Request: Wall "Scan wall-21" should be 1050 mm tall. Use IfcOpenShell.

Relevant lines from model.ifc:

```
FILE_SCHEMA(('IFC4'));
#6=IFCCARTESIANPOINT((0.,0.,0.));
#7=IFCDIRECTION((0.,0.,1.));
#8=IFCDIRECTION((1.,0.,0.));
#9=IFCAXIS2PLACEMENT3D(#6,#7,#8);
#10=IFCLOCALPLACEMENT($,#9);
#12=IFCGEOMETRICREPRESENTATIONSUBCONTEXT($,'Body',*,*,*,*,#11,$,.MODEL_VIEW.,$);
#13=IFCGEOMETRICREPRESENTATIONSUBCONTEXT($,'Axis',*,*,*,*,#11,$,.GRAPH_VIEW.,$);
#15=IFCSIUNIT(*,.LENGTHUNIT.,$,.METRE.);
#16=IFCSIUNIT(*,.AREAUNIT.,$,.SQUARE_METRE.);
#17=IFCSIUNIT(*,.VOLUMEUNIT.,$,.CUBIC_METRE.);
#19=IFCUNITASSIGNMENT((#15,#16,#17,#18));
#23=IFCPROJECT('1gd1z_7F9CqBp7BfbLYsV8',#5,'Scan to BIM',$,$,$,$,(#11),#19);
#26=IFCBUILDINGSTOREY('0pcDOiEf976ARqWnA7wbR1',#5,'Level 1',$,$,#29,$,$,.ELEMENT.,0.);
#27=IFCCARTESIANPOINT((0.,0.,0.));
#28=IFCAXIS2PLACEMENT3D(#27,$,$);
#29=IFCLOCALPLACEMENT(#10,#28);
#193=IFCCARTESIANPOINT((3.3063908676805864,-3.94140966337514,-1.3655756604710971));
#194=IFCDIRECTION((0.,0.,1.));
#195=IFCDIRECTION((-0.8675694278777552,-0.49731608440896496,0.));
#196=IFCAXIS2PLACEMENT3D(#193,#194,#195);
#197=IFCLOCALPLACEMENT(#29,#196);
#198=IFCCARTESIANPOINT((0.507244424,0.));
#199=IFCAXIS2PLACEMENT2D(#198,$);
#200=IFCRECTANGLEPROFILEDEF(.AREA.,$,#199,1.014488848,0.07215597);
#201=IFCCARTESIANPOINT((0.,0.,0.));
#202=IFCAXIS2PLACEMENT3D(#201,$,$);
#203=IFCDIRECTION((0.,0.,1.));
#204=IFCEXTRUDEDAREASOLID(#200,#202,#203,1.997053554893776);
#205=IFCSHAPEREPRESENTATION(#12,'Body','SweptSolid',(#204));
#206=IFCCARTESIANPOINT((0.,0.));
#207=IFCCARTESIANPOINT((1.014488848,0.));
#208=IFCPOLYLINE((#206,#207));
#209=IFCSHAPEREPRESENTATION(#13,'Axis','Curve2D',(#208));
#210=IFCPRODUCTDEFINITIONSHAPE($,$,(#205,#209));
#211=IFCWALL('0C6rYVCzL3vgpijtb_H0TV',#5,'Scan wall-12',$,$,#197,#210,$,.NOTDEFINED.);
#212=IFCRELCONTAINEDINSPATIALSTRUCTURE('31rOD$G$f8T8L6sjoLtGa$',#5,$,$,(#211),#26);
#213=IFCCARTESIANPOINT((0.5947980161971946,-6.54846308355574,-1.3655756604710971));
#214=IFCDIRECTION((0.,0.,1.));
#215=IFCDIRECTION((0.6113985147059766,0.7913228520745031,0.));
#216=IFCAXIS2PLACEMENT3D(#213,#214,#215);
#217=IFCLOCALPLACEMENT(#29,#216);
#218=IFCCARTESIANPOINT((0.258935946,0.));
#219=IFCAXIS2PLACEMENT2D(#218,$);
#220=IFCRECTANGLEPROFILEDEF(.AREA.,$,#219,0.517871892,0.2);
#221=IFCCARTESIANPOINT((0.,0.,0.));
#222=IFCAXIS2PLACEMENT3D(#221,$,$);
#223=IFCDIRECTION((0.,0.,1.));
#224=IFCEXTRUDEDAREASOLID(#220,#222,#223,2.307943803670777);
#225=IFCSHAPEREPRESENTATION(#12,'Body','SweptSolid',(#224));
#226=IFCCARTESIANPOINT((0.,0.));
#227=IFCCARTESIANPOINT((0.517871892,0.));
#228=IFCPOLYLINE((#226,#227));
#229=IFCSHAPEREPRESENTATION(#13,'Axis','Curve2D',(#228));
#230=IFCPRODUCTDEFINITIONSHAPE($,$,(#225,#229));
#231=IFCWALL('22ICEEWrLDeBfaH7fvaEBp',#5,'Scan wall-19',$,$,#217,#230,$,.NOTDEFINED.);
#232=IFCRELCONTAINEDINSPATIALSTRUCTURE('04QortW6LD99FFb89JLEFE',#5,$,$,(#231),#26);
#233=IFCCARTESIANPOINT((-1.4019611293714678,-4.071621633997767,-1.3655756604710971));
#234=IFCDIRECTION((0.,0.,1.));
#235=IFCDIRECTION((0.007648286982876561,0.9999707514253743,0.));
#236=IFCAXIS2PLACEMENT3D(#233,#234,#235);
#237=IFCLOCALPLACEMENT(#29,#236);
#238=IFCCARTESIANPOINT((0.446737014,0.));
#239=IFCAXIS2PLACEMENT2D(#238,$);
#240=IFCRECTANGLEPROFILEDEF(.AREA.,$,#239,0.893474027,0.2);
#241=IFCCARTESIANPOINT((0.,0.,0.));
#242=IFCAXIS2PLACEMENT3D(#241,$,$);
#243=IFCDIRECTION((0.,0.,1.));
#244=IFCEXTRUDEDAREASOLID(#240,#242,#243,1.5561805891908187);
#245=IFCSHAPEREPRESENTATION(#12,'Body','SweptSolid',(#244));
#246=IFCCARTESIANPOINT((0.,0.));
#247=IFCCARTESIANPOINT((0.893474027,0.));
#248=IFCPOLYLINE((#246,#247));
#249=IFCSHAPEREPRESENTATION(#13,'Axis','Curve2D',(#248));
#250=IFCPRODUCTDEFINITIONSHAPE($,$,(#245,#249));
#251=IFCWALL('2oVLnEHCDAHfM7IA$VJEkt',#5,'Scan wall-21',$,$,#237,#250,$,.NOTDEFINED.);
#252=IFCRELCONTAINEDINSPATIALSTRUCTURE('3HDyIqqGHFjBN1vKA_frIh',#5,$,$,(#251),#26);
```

```python
import ifcopenshell
import ifcopenshell.geom
import ifcopenshell.util.shape
import ifcopenshell.util.unit

model = ifcopenshell.open("model.ifc")
unit_scale = ifcopenshell.util.unit.calculate_unit_scale(model)
settings = ifcopenshell.geom.settings()


def volume(element):
    """Net volume in cubic metres, openings subtracted."""
    shape = ifcopenshell.geom.create_shape(settings, element)
    return ifcopenshell.util.shape.get_volume(shape.geometry)


wall = model.by_guid("2oVLnEHCDAHfM7IA$VJEkt")
before = volume(wall)

body = next(r for r in wall.Representation.Representations if r.RepresentationIdentifier == "Body")
solid = body.Items[0]
old_height = solid.Depth
solid.Depth = 1.05 / unit_scale
after = volume(wall)

print(f"height {old_height:g} -> {solid.Depth:g}, volume {before:.3f} -> {after:.3f} m3")

model.write("model_edited.ifc")
```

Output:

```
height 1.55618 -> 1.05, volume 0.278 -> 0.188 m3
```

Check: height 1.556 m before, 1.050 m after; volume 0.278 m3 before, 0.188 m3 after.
